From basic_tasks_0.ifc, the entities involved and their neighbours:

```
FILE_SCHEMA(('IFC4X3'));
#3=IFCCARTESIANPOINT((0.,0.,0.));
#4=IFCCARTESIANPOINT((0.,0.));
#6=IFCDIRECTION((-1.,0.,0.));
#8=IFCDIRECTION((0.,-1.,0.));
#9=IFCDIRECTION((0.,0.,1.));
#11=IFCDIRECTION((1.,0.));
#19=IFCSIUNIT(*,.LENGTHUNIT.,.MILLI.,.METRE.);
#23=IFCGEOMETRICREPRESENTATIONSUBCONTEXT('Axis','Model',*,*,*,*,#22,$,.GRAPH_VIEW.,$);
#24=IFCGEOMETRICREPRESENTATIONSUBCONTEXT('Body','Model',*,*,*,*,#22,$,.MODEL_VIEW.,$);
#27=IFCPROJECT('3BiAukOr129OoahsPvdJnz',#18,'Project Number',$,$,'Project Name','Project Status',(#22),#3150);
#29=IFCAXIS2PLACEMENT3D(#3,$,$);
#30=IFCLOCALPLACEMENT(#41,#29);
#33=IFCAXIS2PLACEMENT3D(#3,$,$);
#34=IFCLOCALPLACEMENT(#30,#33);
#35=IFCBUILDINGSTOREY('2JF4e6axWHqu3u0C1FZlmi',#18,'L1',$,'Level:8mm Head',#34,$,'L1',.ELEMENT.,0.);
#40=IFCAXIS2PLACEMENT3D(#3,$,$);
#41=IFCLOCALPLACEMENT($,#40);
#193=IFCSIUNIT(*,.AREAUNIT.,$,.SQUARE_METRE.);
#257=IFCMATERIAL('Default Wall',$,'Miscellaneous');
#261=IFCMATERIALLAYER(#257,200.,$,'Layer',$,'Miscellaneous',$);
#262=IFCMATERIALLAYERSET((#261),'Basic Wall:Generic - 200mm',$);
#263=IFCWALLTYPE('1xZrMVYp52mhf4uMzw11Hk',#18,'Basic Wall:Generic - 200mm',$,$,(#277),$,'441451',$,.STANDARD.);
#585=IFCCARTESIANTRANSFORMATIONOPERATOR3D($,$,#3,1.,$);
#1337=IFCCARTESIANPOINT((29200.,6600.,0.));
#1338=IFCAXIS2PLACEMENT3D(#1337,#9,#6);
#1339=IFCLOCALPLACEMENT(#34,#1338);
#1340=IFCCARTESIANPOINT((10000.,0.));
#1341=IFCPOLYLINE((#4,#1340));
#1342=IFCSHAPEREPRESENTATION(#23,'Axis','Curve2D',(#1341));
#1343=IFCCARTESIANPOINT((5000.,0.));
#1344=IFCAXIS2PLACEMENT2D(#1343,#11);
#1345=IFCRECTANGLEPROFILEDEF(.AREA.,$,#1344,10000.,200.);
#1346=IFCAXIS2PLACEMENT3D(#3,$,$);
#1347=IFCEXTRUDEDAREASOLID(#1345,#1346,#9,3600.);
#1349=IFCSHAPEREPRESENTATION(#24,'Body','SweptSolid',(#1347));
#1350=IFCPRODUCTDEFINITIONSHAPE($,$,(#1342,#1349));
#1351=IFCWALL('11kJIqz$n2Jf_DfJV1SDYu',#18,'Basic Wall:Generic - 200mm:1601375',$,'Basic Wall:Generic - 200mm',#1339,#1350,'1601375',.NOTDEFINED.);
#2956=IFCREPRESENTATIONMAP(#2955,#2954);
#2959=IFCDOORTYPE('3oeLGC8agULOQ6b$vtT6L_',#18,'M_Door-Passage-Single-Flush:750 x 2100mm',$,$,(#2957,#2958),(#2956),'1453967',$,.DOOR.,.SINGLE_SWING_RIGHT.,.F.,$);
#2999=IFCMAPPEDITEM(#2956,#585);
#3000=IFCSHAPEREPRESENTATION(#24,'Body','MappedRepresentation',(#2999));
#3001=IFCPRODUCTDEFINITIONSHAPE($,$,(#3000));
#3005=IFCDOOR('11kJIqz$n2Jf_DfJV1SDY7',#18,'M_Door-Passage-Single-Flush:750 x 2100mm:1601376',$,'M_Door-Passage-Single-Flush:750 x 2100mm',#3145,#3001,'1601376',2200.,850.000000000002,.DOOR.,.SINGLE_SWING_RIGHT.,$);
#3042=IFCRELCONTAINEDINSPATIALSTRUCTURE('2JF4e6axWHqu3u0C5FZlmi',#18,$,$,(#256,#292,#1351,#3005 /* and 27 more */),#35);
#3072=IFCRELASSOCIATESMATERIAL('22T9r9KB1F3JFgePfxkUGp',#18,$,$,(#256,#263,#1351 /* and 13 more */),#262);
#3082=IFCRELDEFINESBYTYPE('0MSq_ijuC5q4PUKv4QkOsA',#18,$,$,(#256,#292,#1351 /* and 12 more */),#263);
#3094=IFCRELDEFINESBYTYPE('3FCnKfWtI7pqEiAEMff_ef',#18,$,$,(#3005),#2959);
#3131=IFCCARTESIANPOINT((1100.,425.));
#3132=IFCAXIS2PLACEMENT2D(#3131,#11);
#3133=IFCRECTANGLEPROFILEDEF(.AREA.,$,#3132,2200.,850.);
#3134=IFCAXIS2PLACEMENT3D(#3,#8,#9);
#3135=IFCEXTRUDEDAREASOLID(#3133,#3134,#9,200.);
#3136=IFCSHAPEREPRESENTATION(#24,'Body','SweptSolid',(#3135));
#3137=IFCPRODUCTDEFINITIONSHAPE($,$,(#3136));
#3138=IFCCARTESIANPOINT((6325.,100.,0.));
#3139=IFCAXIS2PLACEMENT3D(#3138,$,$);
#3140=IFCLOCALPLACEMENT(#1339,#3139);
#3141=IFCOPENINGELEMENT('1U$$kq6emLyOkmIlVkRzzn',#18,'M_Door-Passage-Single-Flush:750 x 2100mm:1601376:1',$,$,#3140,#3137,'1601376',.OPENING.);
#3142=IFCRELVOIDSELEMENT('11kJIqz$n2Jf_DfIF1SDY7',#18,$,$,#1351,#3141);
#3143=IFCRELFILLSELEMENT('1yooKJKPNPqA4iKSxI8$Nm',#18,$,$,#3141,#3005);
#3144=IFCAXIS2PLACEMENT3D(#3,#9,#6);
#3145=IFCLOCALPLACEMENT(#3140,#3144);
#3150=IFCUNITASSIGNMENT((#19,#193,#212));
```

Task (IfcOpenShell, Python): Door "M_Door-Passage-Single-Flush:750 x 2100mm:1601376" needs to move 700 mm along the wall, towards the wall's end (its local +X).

```python
import ifcopenshell
import ifcopenshell.api.geometry
import ifcopenshell.util.placement
import ifcopenshell.util.unit

model = ifcopenshell.open("basic_tasks_0.ifc")
unit_scale = ifcopenshell.util.unit.calculate_unit_scale(model)

door = model.by_guid("11kJIqz$n2Jf_DfJV1SDY7")
opening = door.FillsVoids[0].RelatingOpeningElement
wall = opening.VoidsElements[0].RelatingBuildingElement

wall_matrix = ifcopenshell.util.placement.get_local_placement(wall.ObjectPlacement)
shift = wall_matrix[:3, 0] * 0.7 / unit_scale
before = ifcopenshell.util.placement.get_local_placement(door.ObjectPlacement)[:3, 3].copy()

# The door is placed relative to its opening, so it follows when the opening moves.
matrix = ifcopenshell.util.placement.get_local_placement(opening.ObjectPlacement)
matrix[:3, 3] += shift
ifcopenshell.api.geometry.edit_object_placement(
    model, product=opening, matrix=matrix, is_si=False, should_transform_children=True
)

after = ifcopenshell.util.placement.get_local_placement(door.ObjectPlacement)[:3, 3]
print("door moved by", (after - before).round(3) + 0.0)

model.write("basic_tasks_0_edited.ifc")
```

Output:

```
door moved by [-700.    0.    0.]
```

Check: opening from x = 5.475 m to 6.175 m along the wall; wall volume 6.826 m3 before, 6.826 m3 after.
